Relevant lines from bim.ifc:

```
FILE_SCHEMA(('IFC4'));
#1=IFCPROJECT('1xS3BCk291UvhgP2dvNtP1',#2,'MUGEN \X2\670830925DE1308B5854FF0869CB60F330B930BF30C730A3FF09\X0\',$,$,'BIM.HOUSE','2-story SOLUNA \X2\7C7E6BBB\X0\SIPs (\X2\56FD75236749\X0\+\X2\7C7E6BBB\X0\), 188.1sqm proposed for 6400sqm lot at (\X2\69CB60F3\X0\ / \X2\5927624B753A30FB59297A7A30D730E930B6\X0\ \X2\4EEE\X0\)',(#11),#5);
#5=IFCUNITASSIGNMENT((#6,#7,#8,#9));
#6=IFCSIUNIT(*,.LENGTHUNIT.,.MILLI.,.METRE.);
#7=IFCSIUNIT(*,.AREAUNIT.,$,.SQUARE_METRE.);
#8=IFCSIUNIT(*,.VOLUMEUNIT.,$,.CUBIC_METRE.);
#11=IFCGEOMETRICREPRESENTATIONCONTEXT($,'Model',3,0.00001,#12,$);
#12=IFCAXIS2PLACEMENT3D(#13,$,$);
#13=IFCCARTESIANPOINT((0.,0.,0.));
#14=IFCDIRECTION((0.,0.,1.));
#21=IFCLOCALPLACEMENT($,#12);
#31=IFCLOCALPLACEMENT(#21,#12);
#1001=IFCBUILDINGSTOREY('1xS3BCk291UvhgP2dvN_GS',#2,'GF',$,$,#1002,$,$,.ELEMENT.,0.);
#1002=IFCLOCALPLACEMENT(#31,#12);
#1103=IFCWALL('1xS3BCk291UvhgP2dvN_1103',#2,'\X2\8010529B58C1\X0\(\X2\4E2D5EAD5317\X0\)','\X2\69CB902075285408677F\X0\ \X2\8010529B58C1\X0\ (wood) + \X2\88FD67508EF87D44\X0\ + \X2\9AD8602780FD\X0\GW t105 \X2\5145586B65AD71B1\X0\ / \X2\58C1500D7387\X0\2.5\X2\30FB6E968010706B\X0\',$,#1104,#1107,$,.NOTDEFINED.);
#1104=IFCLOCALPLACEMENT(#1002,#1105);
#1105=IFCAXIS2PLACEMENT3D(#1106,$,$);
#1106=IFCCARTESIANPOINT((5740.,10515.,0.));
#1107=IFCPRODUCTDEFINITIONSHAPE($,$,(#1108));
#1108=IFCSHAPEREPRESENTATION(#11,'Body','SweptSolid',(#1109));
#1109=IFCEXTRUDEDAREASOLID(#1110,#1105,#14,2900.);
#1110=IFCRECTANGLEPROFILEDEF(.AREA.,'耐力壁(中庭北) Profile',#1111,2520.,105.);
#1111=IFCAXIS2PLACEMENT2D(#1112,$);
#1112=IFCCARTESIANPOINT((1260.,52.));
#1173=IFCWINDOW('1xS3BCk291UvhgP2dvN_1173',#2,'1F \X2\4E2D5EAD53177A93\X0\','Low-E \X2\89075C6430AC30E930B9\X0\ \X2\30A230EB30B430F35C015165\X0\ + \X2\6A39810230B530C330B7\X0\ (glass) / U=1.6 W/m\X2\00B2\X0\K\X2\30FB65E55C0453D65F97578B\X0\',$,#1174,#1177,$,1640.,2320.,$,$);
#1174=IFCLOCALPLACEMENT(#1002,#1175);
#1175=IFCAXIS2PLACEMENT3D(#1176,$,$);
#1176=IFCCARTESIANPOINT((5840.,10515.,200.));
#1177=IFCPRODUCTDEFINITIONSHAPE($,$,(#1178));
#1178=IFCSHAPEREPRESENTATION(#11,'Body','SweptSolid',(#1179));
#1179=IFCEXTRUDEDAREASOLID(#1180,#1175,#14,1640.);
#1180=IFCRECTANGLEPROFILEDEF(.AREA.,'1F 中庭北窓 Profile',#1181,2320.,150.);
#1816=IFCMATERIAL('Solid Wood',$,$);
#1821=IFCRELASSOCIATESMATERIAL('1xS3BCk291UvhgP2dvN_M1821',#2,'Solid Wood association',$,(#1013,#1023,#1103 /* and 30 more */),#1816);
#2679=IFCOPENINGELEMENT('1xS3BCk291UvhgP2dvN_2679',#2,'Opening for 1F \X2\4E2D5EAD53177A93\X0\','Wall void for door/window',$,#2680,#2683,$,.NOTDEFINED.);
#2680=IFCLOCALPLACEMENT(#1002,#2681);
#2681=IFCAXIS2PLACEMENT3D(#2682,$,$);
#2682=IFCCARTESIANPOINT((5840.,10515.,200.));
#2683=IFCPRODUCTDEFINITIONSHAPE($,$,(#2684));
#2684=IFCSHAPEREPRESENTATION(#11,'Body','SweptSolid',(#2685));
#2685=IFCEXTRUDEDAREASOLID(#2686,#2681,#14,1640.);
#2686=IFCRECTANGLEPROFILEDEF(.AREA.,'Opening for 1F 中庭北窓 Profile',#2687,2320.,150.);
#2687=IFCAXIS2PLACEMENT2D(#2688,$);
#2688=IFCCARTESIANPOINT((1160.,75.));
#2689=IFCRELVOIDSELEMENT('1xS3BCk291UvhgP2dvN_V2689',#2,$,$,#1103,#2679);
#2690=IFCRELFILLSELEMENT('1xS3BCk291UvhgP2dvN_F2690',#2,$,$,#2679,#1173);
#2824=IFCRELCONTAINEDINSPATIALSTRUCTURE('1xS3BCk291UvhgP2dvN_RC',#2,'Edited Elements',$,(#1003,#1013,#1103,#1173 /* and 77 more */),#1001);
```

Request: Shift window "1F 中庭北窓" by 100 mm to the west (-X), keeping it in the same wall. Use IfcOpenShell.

```python
import ifcopenshell
import ifcopenshell.api.geometry
import ifcopenshell.util.placement
import ifcopenshell.util.unit

model = ifcopenshell.open("bim.ifc")
unit_scale = ifcopenshell.util.unit.calculate_unit_scale(model)

window = model.by_guid("1xS3BCk291UvhgP2dvN_1173")
opening = window.FillsVoids[0].RelatingOpeningElement
wall = opening.VoidsElements[0].RelatingBuildingElement

wall_matrix = ifcopenshell.util.placement.get_local_placement(wall.ObjectPlacement)
shift = wall_matrix[:3, 0] * -0.1 / unit_scale
before = ifcopenshell.util.placement.get_local_placement(window.ObjectPlacement)[:3, 3].copy()

# The window is not placed relative to its opening, so move both.
for product in (opening, window):
    matrix = ifcopenshell.util.placement.get_local_placement(product.ObjectPlacement)
    matrix[:3, 3] += shift
    ifcopenshell.api.geometry.edit_object_placement(model, product=product, matrix=matrix, is_si=False)

after = ifcopenshell.util.placement.get_local_placement(window.ObjectPlacement)[:3, 3]
print("window moved by", (after - before).round(3) + 0.0)

model.write("bim-out.ifc")
```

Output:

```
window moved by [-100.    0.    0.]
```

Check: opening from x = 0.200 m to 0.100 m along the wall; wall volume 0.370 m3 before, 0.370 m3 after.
